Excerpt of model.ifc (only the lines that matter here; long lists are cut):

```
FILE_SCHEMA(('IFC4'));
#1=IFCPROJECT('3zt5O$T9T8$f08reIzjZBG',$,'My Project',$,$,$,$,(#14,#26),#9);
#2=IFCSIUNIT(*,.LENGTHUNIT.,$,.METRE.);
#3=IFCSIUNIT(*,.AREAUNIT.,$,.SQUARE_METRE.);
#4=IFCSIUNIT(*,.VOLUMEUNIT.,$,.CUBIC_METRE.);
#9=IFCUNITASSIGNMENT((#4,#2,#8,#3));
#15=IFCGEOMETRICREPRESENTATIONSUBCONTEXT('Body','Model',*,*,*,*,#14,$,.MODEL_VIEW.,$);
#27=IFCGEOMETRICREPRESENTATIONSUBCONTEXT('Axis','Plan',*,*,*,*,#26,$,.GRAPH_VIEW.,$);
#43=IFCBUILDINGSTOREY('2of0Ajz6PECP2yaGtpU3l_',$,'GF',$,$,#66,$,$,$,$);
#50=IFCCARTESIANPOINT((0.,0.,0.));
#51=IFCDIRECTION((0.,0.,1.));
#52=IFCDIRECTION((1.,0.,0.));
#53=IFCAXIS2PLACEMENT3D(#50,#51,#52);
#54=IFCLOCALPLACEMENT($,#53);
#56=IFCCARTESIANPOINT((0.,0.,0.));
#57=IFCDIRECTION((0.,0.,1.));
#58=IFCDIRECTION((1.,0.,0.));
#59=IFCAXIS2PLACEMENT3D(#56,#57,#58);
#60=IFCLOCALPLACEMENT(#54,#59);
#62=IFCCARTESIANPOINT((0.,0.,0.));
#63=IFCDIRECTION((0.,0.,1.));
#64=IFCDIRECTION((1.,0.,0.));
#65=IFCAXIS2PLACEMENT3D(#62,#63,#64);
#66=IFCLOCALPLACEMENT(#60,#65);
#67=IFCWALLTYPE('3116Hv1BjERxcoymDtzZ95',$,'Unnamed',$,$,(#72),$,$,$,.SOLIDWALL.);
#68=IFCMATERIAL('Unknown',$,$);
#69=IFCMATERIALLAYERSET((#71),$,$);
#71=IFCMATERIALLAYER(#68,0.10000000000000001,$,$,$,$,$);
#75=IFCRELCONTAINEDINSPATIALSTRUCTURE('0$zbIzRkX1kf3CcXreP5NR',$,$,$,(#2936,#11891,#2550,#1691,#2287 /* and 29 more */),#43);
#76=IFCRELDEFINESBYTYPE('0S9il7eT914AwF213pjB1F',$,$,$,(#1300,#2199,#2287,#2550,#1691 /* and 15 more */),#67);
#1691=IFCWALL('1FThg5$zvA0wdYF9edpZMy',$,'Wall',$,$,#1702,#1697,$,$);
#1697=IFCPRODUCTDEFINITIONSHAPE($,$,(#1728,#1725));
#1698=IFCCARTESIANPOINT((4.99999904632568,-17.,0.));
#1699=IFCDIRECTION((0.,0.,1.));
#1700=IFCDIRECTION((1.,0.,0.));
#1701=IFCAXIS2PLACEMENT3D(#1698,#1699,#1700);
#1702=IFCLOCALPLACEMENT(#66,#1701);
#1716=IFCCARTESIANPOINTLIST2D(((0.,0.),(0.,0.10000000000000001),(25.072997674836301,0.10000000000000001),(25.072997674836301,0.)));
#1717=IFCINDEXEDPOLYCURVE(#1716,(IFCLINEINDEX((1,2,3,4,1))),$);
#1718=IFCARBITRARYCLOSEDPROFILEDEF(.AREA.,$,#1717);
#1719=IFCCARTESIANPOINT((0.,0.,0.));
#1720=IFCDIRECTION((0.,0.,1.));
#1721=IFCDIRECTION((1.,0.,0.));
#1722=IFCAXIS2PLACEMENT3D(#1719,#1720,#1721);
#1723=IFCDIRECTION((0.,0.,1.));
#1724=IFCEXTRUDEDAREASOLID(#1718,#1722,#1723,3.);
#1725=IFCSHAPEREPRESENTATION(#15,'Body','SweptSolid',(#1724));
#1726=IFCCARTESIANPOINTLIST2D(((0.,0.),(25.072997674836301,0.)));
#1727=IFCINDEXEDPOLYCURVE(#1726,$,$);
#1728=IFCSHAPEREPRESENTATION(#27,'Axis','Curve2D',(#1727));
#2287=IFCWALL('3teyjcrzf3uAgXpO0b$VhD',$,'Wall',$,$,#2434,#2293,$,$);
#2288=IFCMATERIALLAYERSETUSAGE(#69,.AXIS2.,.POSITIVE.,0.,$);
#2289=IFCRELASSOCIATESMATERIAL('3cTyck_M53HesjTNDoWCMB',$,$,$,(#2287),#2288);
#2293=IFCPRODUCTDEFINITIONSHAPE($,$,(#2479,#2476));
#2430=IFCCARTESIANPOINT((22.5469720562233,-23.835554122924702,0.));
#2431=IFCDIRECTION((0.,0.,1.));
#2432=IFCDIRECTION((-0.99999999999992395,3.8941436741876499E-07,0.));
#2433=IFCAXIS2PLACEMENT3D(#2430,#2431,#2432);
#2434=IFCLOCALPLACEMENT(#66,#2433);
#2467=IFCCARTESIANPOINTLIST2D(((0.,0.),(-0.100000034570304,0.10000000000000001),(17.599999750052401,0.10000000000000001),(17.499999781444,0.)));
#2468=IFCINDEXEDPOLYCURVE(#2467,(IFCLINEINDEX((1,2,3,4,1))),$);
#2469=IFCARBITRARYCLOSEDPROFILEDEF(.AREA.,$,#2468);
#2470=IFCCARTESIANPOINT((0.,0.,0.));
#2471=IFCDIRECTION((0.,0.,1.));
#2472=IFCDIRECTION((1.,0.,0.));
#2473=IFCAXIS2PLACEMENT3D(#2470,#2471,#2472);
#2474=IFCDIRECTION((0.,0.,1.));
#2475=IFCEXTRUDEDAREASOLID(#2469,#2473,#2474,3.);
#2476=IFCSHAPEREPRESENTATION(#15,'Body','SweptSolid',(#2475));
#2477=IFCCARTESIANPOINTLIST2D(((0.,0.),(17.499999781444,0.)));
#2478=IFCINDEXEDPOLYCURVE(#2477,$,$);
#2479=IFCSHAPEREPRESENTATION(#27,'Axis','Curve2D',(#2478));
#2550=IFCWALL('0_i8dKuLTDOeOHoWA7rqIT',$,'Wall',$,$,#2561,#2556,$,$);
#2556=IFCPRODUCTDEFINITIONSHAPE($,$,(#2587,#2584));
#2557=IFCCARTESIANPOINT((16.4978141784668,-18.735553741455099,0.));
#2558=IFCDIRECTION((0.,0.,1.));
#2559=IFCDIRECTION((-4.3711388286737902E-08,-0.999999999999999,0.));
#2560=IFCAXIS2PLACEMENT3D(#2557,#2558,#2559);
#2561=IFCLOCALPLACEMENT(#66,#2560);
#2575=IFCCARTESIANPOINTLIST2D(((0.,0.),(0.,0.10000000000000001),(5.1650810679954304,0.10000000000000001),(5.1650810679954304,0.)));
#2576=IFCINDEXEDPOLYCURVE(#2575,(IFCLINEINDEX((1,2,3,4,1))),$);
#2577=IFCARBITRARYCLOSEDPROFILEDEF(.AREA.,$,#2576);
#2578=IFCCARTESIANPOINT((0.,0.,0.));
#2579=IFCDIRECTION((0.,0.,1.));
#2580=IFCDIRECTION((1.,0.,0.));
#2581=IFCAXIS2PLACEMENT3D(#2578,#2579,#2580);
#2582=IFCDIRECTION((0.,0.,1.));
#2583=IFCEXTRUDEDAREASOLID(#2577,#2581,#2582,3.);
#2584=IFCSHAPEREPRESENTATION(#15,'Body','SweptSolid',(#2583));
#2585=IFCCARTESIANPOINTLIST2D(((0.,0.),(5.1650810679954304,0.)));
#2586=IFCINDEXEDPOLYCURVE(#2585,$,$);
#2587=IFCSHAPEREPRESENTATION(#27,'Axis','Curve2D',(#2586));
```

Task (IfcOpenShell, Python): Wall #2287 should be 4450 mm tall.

```python
import ifcopenshell
import ifcopenshell.geom
import ifcopenshell.util.representation
import ifcopenshell.util.shape
import ifcopenshell.util.unit

model = ifcopenshell.open("model.ifc")
unit_scale = ifcopenshell.util.unit.calculate_unit_scale(model)
settings = ifcopenshell.geom.settings()


def volume(element):
    """Net volume in cubic metres, openings subtracted."""
    shape = ifcopenshell.geom.create_shape(settings, element)
    return ifcopenshell.util.shape.get_volume(shape.geometry)


wall = model.by_guid("3teyjcrzf3uAgXpO0b$VhD")
before = volume(wall)

body = ifcopenshell.util.representation.get_representation(wall, "Model", "Body")
solid = body.Items[0]
old_height = solid.Depth
solid.Depth = 4.45 / unit_scale
after = volume(wall)

print(f"height {old_height:g} -> {solid.Depth:g}, volume {before:.3f} -> {after:.3f} m3")

model.write("model_v2.ifc")
```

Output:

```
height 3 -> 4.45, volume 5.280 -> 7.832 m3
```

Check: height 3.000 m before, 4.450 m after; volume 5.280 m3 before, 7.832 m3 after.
